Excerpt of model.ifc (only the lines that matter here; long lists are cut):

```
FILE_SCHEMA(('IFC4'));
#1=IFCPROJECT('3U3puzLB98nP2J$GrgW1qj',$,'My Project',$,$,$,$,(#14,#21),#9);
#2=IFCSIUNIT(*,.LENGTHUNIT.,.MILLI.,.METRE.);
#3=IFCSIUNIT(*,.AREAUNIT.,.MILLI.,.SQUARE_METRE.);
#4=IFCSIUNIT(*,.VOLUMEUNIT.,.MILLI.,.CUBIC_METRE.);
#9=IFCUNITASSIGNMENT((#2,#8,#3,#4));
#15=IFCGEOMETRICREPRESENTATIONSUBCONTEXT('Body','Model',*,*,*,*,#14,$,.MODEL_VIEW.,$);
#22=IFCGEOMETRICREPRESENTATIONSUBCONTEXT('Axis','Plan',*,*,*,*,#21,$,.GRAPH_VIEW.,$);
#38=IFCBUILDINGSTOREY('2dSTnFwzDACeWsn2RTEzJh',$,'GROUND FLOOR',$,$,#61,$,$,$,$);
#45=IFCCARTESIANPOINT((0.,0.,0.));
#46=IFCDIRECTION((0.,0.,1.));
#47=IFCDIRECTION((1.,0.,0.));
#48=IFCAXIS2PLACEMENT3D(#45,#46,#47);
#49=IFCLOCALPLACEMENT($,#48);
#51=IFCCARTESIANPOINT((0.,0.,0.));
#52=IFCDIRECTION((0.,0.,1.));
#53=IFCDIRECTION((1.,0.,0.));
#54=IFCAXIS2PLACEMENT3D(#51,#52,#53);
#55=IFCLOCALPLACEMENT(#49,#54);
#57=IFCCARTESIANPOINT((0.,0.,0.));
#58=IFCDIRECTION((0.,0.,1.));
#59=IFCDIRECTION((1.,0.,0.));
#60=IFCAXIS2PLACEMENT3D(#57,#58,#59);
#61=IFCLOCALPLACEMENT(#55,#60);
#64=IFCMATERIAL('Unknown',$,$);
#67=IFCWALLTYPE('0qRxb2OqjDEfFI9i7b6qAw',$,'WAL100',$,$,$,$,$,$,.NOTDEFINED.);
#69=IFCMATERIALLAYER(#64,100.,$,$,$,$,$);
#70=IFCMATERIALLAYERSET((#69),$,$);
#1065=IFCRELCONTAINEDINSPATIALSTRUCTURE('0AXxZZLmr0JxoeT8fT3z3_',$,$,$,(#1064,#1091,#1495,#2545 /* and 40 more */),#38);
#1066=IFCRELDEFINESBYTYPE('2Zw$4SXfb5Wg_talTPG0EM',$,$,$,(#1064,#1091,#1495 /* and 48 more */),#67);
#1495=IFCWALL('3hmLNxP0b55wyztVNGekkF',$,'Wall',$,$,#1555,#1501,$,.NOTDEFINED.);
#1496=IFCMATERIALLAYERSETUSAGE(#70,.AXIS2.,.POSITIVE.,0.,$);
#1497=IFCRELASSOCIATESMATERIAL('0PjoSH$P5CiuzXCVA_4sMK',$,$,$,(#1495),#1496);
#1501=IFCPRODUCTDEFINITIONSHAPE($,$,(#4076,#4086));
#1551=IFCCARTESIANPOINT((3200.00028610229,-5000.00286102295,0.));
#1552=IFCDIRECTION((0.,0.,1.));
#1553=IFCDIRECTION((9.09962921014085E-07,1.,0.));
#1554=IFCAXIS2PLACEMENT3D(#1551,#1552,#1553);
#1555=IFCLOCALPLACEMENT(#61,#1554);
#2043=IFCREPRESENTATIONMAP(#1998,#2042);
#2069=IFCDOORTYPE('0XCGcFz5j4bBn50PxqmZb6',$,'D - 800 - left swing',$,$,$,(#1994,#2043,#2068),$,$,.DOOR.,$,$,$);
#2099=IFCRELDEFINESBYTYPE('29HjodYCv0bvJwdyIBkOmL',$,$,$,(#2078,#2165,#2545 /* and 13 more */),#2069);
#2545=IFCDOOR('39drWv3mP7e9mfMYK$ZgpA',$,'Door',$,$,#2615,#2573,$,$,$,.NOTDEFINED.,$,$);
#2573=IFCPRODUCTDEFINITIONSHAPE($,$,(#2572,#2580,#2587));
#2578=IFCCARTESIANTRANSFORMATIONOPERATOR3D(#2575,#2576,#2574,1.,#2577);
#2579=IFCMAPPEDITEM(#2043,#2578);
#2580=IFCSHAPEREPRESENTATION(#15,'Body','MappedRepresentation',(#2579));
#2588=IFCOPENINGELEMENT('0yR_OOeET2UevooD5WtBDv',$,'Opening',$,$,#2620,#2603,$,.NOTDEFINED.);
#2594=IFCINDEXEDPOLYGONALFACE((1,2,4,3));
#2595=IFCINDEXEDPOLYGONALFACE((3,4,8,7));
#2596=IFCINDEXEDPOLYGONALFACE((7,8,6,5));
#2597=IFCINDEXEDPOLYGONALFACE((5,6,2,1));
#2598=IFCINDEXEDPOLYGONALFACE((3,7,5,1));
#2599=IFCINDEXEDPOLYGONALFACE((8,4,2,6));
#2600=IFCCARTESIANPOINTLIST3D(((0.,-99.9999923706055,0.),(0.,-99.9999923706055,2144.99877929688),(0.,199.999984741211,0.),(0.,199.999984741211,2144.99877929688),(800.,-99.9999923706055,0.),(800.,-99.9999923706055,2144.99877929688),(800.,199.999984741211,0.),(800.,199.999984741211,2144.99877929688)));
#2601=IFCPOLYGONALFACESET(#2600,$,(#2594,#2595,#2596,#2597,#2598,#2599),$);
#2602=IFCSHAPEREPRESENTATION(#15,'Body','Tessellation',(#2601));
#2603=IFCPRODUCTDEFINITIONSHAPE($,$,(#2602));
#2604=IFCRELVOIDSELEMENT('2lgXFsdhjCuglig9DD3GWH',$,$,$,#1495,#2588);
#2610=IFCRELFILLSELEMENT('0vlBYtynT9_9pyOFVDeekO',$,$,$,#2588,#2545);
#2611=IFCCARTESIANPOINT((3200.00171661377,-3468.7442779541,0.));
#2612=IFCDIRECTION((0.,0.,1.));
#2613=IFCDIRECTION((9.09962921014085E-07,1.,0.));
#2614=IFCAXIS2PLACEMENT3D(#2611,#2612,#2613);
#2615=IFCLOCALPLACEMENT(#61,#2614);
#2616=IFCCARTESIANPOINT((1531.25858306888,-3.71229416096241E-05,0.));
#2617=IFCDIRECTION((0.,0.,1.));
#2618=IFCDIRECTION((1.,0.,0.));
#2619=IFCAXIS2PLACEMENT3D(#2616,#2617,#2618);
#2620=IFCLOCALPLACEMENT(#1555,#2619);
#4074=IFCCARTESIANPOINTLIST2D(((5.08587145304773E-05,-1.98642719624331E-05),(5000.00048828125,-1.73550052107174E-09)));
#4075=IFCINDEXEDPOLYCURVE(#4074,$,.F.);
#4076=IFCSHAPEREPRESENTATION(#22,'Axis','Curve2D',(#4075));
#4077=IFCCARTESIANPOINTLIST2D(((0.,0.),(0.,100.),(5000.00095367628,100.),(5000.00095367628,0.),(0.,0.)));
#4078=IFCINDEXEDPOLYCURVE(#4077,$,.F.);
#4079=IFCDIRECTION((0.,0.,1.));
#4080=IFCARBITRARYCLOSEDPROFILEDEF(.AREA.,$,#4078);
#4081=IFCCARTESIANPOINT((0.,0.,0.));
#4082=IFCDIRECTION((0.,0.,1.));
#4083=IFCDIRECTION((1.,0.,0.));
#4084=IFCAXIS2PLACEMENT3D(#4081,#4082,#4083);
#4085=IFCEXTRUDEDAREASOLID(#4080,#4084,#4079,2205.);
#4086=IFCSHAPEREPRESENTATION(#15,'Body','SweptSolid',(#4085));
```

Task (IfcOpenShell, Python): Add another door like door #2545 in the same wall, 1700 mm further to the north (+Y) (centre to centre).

```python
import ifcopenshell
import ifcopenshell.api.feature
import ifcopenshell.api.geometry
import ifcopenshell.api.root
import ifcopenshell.geom
import ifcopenshell.util.element
import ifcopenshell.util.placement
import ifcopenshell.util.shape

model = ifcopenshell.open("model.ifc")
settings = ifcopenshell.geom.settings()


def volume(element):
    """Net volume in cubic metres, openings subtracted."""
    shape = ifcopenshell.geom.create_shape(settings, element)
    return ifcopenshell.util.shape.get_volume(shape.geometry)


door = model.by_guid("39drWv3mP7e9mfMYK$ZgpA")
opening = door.FillsVoids[0].RelatingOpeningElement
wall = opening.VoidsElements[0].RelatingBuildingElement
before = volume(wall)
shift = ifcopenshell.util.placement.get_local_placement(wall.ObjectPlacement)[:3, 0] * 1700.0

# copy_class copies the void relationship, type, container and properties, but no geometry.
new_opening = ifcopenshell.api.root.copy_class(model, product=opening)
new_opening.Representation = ifcopenshell.util.element.copy_deep(
    model, opening.Representation, exclude=["IfcGeometricRepresentationContext", "IfcRepresentationMap"]
)
new_door = ifcopenshell.api.root.copy_class(model, product=door)
new_door.Representation = ifcopenshell.util.element.copy_deep(
    model, door.Representation, exclude=["IfcGeometricRepresentationContext", "IfcRepresentationMap"]
)
ifcopenshell.api.feature.add_filling(model, opening=new_opening, element=new_door)

for old, new in ((opening, new_opening), (door, new_door)):
    matrix = ifcopenshell.util.placement.get_local_placement(old.ObjectPlacement)
    matrix[:3, 3] += shift
    ifcopenshell.api.geometry.edit_object_placement(model, product=new, matrix=matrix, is_si=False)

after = volume(wall)

print(f"wall volume {before:.3f} -> {after:.3f} m3")

model.write("model_v2.ifc")
```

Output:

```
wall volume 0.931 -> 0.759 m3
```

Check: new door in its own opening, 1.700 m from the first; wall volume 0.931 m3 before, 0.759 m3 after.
